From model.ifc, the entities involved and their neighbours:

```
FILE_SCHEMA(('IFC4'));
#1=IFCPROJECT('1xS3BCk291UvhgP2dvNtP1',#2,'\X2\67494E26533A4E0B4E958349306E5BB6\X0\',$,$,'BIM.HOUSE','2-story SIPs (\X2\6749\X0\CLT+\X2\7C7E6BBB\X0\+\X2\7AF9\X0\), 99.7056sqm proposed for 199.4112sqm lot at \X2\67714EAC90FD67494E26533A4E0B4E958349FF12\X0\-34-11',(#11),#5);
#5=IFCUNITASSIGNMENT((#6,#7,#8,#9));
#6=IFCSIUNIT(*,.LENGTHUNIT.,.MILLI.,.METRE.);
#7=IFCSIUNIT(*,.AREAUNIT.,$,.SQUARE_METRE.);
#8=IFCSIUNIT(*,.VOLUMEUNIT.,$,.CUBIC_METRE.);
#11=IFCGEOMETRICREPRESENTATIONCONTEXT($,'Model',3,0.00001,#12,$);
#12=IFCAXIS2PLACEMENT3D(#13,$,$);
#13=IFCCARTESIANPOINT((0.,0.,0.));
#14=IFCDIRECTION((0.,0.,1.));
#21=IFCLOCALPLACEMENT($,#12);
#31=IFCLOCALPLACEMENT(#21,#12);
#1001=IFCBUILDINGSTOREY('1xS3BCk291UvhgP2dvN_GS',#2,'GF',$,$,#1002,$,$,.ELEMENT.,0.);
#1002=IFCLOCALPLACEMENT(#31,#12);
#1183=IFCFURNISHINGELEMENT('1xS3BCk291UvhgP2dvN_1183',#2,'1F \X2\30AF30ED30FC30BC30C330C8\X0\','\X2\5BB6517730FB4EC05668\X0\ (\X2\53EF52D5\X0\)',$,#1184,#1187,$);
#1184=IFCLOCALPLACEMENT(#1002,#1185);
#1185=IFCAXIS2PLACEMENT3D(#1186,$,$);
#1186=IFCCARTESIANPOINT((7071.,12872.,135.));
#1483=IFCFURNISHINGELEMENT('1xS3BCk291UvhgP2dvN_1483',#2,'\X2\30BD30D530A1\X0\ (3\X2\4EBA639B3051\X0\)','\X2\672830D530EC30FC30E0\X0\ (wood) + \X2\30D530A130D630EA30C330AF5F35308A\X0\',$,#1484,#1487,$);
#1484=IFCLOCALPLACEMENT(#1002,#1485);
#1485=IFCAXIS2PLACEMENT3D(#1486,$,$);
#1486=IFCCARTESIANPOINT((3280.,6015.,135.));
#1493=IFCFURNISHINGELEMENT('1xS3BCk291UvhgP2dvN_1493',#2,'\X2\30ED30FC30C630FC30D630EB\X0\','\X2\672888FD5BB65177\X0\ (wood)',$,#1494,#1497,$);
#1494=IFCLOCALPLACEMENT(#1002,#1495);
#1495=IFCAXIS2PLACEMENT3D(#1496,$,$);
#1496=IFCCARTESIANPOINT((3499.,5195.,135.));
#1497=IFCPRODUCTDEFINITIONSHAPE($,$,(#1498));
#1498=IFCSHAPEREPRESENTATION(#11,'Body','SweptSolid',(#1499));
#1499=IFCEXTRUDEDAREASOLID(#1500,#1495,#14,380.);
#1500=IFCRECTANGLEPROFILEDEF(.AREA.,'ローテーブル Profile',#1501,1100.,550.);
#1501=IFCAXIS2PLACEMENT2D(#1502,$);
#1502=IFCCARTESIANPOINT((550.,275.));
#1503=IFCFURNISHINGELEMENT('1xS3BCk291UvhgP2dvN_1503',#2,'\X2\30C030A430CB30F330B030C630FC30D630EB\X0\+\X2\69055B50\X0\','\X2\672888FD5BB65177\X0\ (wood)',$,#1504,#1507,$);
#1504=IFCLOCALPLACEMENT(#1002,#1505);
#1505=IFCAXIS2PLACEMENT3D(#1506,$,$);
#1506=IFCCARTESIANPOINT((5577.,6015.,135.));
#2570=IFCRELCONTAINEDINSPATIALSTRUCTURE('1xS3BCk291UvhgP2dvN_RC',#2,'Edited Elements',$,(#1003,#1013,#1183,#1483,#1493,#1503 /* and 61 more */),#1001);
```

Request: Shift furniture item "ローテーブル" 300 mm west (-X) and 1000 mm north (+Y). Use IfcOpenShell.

```python
import ifcopenshell
import ifcopenshell.api.geometry
import ifcopenshell.util.placement

model = ifcopenshell.open("model.ifc")

item = model.by_guid("1xS3BCk291UvhgP2dvN_1493")
matrix = ifcopenshell.util.placement.get_local_placement(item.ObjectPlacement)
matrix[0, 3] -= 300.0
matrix[1, 3] += 1000.0
ifcopenshell.api.geometry.edit_object_placement(model, product=item, matrix=matrix, is_si=False)

print(ifcopenshell.util.placement.get_local_placement(item.ObjectPlacement).round(3) + 0.0)

model.write("model-out.ifc")
```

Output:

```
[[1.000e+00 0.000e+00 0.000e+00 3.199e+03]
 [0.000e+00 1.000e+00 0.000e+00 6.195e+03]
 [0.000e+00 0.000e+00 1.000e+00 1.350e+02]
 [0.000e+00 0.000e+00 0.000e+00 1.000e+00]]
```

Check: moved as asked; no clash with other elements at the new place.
